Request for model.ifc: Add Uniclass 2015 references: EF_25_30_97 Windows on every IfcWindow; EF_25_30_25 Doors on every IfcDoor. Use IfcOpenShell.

First a look at what the model holds.

```python
import ifcopenshell

model = ifcopenshell.open("model.ifc")
print(model.schema)
print("classifications:", [c.Name for c in model.by_type("IfcClassification")])
for ifc_class in ("IfcDoor", "IfcRoof", "IfcStair", "IfcWall", "IfcWindow"):
    print(ifc_class, len(model.by_type(ifc_class)))
```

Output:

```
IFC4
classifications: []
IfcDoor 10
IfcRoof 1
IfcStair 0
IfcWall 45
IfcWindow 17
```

```python
import ifcopenshell
import ifcopenshell.api.classification

model = ifcopenshell.open("model.ifc")

system = ifcopenshell.api.classification.add_classification(model, classification="Uniclass 2015")

codes = {
    "IfcWindow": ("EF_25_30_97", "Windows"),
    "IfcDoor": ("EF_25_30_25", "Doors"),
}
for ifc_class, (code, name) in codes.items():
    products = model.by_type(ifc_class)
    ifcopenshell.api.classification.add_reference(
        model, products=products, classification=system, identification=code, name=name
    )
    print(code, len(products))

model.write("model_v2.ifc")
```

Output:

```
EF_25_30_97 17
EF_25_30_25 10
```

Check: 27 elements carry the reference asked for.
